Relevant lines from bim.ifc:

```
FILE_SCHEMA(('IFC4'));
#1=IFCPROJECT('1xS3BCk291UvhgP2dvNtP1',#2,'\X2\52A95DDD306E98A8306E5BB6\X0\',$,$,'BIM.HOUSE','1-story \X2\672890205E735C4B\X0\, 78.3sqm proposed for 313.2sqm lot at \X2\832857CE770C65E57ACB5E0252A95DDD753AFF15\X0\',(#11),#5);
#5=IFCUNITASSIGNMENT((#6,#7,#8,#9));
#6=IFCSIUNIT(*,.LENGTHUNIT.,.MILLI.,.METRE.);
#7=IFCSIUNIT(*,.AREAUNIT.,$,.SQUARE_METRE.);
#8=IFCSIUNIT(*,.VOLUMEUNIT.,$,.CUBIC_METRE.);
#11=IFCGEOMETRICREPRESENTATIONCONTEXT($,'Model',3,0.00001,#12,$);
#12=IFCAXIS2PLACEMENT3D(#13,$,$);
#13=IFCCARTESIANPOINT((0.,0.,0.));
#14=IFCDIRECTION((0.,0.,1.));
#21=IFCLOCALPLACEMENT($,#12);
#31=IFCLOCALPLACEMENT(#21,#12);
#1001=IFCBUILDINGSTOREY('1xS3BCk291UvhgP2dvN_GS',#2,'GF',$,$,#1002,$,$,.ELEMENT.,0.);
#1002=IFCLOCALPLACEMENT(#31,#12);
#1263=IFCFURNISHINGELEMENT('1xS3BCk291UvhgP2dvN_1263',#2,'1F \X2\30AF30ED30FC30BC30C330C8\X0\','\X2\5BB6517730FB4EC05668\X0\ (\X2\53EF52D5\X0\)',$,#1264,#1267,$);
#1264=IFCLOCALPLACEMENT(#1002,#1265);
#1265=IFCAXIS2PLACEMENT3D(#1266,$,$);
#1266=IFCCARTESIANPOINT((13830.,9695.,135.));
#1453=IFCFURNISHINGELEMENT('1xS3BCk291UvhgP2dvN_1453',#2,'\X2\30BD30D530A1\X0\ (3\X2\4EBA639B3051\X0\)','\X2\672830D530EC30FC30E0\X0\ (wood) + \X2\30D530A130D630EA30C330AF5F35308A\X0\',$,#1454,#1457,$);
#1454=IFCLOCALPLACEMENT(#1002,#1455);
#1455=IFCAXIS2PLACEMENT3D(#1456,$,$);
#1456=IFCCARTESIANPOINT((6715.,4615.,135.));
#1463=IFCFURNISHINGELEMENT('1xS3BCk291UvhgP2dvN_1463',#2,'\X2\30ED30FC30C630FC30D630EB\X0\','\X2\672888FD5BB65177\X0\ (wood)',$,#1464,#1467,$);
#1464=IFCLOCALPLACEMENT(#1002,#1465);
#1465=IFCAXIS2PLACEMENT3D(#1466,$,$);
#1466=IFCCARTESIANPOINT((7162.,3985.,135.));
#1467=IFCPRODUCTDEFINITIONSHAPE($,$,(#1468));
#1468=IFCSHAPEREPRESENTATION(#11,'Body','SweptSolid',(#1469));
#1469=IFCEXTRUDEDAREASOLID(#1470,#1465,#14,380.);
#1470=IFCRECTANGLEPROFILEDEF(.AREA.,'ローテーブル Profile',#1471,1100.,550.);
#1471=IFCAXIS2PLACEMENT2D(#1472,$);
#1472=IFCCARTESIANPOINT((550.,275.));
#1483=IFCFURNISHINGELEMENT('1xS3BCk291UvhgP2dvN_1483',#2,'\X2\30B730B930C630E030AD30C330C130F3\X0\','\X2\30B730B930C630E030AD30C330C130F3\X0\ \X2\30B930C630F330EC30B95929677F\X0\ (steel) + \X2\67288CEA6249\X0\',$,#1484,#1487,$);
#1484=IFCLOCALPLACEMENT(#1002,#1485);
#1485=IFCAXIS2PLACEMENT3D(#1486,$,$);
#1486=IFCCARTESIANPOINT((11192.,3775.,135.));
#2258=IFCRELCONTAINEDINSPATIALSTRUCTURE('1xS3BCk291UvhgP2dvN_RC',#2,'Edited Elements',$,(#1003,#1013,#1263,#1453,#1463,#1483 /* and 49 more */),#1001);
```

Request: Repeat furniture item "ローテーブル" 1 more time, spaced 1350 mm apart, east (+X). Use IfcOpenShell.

```python
import numpy as np
import ifcopenshell
import ifcopenshell.api.geometry
import ifcopenshell.api.root
import ifcopenshell.util.element
import ifcopenshell.util.placement

model = ifcopenshell.open("bim.ifc")


def reuse_history(source, copy):
    """copy_class also copies each property set's owner history, people and application; keep the originals."""
    for rel in copy.IsDefinedBy:
        if rel.is_a("IfcRelDefinesByProperties") and (history := rel.RelatingPropertyDefinition.OwnerHistory):
            rel.RelatingPropertyDefinition.OwnerHistory = source.OwnerHistory
            ifcopenshell.util.element.remove_deep2(model, history)


source = model.by_guid("1xS3BCk291UvhgP2dvN_1463")
base = ifcopenshell.util.placement.get_local_placement(source.ObjectPlacement)
step = np.array([1.0, 0.0, 0.0]) * 1350.0

for i in range(1, 2):
    copy = ifcopenshell.api.root.copy_class(model, product=source)
    copy.Representation = ifcopenshell.util.element.copy_deep(
        model, source.Representation, exclude=["IfcGeometricRepresentationContext", "IfcRepresentationMap"]
    )
    reuse_history(source, copy)
    matrix = base.copy()
    matrix[:3, 3] += i * step
    print("added at", matrix[:3, 3].round(3) + 0.0)
    ifcopenshell.api.geometry.edit_object_placement(model, product=copy, matrix=matrix, is_si=False)

model.write("bim-out.ifc")
```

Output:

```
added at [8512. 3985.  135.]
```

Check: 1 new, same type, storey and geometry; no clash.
